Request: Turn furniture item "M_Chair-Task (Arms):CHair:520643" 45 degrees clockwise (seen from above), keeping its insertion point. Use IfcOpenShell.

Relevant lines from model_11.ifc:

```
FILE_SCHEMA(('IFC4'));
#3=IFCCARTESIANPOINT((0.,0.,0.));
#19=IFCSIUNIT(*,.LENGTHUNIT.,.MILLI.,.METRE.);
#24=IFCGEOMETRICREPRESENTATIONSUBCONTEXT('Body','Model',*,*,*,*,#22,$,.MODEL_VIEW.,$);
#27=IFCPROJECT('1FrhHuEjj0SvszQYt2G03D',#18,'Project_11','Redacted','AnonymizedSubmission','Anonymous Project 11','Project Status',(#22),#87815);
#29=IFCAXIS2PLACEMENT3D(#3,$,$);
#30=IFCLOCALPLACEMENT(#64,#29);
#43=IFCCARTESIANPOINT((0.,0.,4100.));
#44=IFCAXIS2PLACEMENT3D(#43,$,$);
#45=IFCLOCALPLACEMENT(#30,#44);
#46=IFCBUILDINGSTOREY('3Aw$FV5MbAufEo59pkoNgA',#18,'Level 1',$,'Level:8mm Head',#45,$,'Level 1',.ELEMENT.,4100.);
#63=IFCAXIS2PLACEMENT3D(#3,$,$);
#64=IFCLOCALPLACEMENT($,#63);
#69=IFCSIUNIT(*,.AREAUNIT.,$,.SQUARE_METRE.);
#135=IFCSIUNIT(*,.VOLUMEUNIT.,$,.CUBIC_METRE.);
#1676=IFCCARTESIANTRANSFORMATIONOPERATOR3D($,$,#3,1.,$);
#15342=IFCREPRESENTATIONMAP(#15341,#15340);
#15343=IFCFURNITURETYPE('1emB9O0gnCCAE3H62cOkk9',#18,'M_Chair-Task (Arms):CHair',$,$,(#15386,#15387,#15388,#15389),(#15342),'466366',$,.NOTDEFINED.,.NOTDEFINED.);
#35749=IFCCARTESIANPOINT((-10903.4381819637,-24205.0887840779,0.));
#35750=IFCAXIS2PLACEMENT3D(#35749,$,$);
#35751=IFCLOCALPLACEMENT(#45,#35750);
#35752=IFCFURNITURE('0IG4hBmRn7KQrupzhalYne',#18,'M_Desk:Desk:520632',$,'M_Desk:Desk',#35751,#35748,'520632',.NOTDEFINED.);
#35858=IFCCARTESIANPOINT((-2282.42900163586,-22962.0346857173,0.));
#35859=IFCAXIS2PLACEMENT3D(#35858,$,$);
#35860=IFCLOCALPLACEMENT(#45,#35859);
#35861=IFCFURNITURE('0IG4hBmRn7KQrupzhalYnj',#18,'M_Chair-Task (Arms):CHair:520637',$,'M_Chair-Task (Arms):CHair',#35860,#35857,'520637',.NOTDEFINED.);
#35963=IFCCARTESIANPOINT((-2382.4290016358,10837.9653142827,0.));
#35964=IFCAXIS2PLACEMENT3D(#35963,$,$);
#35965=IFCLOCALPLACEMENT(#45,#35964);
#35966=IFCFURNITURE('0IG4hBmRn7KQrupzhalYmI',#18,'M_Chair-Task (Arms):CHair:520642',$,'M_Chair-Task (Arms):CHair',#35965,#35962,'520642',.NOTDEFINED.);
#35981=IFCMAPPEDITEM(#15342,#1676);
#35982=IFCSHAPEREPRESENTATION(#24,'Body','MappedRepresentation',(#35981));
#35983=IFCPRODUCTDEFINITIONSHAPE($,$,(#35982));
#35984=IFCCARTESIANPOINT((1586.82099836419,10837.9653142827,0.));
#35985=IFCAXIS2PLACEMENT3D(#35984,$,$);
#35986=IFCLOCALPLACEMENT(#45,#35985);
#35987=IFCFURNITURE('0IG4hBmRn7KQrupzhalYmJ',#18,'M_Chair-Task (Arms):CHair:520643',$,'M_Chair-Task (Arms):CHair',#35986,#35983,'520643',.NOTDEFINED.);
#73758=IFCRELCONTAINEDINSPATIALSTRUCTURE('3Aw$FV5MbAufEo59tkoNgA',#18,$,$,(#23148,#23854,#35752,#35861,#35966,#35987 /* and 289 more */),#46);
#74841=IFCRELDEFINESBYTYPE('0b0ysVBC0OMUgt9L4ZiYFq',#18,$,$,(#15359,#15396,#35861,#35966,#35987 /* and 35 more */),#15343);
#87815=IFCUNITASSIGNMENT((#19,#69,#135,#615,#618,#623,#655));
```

```python
import ifcopenshell
import ifcopenshell.api.geometry
import ifcopenshell.util.placement

model = ifcopenshell.open("model_11.ifc")

item = model.by_guid("0IG4hBmRn7KQrupzhalYmJ")
matrix = ifcopenshell.util.placement.get_local_placement(item.ObjectPlacement)
matrix = matrix @ ifcopenshell.util.placement.rotation(-45, "Z")
ifcopenshell.api.geometry.edit_object_placement(model, product=item, matrix=matrix, is_si=False)

print(ifcopenshell.util.placement.get_local_placement(item.ObjectPlacement).round(3) + 0.0)

model.write("model_11_rev.ifc")
```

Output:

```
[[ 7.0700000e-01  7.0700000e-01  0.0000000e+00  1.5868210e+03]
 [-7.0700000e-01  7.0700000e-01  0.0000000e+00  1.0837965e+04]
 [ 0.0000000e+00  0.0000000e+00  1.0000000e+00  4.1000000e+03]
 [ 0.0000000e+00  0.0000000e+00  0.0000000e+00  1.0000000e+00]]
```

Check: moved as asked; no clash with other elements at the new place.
